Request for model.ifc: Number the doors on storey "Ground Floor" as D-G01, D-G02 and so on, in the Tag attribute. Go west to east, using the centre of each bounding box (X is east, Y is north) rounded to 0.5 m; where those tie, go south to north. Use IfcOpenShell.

First a look at what the model holds.

```python
import ifcopenshell
import ifcopenshell.util.element
import ifcopenshell.util.placement

model = ifcopenshell.open("model.ifc")
print(model.schema)
storey = next(s for s in model.by_type("IfcBuildingStorey") if s.Name == "Ground Floor")
doors = [e for e in ifcopenshell.util.element.get_decomposition(storey) if e.is_a("IfcDoor")]
for e in sorted(doors, key=lambda e: e.id()):
    origin = ifcopenshell.util.placement.get_local_placement(e.ObjectPlacement)[:3, 3]
    print(e.id(), e.Tag, e.Name, origin.round(2) + 0.0, sep=" | ")
```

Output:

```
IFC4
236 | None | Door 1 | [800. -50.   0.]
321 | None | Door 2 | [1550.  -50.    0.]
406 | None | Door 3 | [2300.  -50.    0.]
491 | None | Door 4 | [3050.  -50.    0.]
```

```python
import ifcopenshell
import ifcopenshell.geom
import ifcopenshell.util.element
import ifcopenshell.util.shape

model = ifcopenshell.open("model.ifc")
settings = ifcopenshell.geom.settings()
settings.set("use-world-coords", True)


def centre(element):
    shape = ifcopenshell.geom.create_shape(settings, element)
    return ifcopenshell.util.shape.get_bbox_centroid(shape.geometry)


storey = next(s for s in model.by_type("IfcBuildingStorey") if s.Name == "Ground Floor")
doors = [e for e in ifcopenshell.util.element.get_decomposition(storey) if e.is_a("IfcDoor")]

# Insertion points can sit at a corner or the storey origin, so sort by the geometry (in metres).
centres = {e: centre(e) for e in doors}
doors.sort(key=lambda e: (round(centres[e][0] / 0.5), centres[e][1]))

for i, e in enumerate(doors, start=1):
    number = f"D-G{i:02d}"
    e.Tag = number
    print(e.id(), number)

model.write("model-out.ifc")
```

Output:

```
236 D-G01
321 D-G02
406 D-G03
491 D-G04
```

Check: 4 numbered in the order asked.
